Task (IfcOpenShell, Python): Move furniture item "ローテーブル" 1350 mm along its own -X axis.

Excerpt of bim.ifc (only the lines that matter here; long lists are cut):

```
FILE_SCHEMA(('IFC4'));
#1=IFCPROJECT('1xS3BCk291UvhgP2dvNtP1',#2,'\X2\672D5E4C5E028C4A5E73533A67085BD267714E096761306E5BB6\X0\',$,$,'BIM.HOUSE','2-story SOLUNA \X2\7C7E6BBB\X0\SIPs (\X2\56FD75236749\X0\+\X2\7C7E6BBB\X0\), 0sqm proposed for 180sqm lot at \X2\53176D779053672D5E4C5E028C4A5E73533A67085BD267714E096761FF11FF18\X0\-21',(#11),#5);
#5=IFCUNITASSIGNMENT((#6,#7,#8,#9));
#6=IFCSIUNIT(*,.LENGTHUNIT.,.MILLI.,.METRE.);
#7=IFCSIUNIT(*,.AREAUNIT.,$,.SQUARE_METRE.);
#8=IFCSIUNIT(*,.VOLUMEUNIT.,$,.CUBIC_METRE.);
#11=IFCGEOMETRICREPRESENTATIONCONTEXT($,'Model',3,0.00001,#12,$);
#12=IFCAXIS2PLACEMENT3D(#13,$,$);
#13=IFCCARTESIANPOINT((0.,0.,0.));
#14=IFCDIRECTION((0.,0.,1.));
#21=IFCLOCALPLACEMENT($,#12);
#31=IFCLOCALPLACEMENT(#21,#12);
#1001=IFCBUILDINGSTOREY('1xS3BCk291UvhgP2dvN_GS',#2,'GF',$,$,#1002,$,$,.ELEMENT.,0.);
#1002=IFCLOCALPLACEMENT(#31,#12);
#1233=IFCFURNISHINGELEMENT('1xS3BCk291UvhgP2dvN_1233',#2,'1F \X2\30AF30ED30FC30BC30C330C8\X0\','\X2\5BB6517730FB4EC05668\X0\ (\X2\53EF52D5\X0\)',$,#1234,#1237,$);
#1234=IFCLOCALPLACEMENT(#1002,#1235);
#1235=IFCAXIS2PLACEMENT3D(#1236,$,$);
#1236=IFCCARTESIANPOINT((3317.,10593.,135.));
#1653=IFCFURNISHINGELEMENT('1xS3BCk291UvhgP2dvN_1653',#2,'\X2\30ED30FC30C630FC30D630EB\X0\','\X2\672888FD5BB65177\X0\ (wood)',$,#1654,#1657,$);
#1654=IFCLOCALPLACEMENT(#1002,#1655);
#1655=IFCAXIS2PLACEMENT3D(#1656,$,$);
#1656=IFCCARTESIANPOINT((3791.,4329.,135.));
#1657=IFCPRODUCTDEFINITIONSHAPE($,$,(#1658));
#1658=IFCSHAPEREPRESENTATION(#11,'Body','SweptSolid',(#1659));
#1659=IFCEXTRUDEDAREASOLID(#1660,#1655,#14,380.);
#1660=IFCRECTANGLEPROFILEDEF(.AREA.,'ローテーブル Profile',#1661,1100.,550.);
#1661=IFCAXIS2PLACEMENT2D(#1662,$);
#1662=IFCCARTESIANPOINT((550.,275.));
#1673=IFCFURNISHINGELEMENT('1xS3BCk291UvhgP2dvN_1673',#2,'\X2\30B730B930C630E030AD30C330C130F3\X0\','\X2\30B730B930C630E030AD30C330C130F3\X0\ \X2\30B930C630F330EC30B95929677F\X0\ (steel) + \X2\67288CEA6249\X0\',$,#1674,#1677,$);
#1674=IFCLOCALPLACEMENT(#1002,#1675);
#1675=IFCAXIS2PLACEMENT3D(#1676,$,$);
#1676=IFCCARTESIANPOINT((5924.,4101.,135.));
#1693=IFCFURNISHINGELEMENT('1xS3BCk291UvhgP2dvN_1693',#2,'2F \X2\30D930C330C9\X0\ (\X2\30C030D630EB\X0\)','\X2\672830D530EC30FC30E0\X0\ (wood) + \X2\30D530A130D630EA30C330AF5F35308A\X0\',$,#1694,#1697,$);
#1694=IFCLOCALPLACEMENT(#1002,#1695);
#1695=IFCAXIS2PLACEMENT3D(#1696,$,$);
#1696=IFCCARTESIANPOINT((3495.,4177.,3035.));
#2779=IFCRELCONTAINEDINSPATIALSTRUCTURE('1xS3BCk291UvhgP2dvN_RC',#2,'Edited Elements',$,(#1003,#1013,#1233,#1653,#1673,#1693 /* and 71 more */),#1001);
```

```python
import ifcopenshell
import ifcopenshell.api.geometry
import ifcopenshell.util.placement
import ifcopenshell.util.unit

model = ifcopenshell.open("bim.ifc")
unit_scale = ifcopenshell.util.unit.calculate_unit_scale(model)

item = model.by_guid("1xS3BCk291UvhgP2dvN_1653")
matrix = ifcopenshell.util.placement.get_local_placement(item.ObjectPlacement)
matrix[:3, 3] -= matrix[:3, 0] * 1.35 / unit_scale
ifcopenshell.api.geometry.edit_object_placement(model, product=item, matrix=matrix, is_si=False)

print(ifcopenshell.util.placement.get_local_placement(item.ObjectPlacement).round(3) + 0.0)

model.write("bim_v2.ifc")
```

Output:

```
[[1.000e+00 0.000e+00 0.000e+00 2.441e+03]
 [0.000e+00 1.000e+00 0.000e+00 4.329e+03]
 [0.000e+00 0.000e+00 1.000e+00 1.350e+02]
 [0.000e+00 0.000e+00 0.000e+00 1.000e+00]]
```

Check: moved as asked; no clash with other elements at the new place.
